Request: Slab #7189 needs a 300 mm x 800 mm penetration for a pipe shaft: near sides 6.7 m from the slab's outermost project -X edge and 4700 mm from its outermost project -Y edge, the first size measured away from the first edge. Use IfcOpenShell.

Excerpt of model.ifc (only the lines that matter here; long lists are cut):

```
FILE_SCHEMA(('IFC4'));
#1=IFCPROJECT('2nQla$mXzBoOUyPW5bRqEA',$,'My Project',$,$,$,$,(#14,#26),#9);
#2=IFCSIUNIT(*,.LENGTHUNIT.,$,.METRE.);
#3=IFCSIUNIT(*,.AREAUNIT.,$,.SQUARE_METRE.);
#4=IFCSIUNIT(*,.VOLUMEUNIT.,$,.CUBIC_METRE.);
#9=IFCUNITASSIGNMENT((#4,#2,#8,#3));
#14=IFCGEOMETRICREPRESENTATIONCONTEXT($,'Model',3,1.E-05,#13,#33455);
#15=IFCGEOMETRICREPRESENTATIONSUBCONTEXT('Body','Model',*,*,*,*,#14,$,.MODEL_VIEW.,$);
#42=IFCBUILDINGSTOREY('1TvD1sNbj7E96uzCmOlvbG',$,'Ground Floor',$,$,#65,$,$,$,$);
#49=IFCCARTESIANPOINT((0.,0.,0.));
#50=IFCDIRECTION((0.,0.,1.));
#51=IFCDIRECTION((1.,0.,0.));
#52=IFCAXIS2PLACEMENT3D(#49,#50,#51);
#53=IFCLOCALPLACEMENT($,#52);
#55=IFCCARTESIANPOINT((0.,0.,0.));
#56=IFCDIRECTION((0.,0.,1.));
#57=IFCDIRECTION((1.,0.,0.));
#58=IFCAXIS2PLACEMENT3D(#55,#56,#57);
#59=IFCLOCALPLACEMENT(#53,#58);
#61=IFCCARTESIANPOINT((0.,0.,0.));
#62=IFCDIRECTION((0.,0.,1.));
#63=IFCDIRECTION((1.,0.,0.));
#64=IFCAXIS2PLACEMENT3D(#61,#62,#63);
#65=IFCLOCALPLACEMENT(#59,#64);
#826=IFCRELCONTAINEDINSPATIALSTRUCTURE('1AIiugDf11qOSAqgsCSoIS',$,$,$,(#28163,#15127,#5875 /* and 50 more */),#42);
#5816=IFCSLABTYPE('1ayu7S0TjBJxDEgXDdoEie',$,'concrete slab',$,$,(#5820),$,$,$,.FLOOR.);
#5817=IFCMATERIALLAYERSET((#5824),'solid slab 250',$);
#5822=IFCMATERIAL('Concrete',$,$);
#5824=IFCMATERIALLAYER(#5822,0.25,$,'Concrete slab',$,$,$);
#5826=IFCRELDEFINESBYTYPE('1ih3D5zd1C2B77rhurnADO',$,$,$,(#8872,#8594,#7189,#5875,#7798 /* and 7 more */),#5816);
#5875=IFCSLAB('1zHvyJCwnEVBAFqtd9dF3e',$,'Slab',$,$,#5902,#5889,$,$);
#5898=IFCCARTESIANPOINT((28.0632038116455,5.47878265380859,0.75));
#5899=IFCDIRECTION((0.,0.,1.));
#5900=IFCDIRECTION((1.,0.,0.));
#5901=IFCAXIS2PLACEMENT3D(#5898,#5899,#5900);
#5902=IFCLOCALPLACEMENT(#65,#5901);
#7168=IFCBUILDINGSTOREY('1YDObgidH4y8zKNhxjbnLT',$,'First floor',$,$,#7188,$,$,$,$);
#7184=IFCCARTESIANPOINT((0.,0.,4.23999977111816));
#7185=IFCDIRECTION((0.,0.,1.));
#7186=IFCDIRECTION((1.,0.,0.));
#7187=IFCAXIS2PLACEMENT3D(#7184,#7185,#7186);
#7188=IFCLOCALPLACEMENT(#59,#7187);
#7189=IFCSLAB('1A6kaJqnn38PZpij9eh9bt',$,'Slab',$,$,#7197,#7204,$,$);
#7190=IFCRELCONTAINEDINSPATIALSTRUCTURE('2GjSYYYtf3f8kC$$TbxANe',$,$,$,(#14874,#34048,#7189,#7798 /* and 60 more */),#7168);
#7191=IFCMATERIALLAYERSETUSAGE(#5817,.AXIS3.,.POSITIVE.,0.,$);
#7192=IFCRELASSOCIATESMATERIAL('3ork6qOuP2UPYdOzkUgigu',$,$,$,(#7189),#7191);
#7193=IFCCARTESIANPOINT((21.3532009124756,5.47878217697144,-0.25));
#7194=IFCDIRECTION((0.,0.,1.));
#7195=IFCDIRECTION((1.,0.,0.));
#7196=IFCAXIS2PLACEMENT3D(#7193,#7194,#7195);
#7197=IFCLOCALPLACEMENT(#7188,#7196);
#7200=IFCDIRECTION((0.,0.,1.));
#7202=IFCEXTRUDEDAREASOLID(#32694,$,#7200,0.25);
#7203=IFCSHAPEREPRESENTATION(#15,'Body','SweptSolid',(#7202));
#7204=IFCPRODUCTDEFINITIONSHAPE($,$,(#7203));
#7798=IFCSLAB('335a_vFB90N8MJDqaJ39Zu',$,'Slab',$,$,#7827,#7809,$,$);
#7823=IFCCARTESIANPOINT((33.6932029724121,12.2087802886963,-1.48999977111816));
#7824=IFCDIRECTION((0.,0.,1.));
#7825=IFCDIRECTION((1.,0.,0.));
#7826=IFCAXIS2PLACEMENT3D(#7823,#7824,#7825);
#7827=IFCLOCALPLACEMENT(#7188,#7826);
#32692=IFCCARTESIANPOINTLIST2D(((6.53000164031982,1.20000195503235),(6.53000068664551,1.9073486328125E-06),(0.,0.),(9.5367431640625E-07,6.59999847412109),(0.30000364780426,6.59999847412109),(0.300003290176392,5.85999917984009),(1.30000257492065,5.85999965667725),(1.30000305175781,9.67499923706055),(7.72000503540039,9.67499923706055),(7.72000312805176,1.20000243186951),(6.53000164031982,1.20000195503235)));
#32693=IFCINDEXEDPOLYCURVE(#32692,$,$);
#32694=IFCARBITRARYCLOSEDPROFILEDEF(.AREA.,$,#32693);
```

```python
import numpy as np
import ifcopenshell
import ifcopenshell.api.feature
import ifcopenshell.api.geometry
import ifcopenshell.api.root
import ifcopenshell.geom
import ifcopenshell.util.placement
import ifcopenshell.util.representation
import ifcopenshell.util.shape
import ifcopenshell.util.unit

model = ifcopenshell.open("model.ifc")
unit_scale = ifcopenshell.util.unit.calculate_unit_scale(model)
settings = ifcopenshell.geom.settings()


def volume(element):
    """Net volume in cubic metres, openings subtracted."""
    shape = ifcopenshell.geom.create_shape(settings, element)
    return ifcopenshell.util.shape.get_volume(shape.geometry)


slab = model.by_id(7189)
before = volume(slab)

# Extent in the slab's own axes, in metres. The edges named are its -X and -Y sides.
slab_shape = ifcopenshell.geom.create_shape(settings, slab)
vertices = ifcopenshell.util.shape.get_vertices(slab_shape.geometry)
x_min, y_min, bottom = vertices.min(axis=0)
top = vertices[:, 2].max()

opening = ifcopenshell.api.root.create_entity(model, ifc_class="IfcOpeningElement", name="Pipe shaft opening", predefined_type="OPENING")
context = ifcopenshell.util.representation.get_context(model, "Model", "Body", "MODEL_VIEW")
width, depth = 0.3, 0.8
outline = [(0.0, 0.0), (width, 0.0), (width, depth), (0.0, depth), (0.0, 0.0)]
# Overshoot both faces by 50 mm so the cut is clean.
shape = ifcopenshell.api.geometry.add_slab_representation(
    model, context=context, depth=top - bottom + 0.1, polyline=outline
)
ifcopenshell.api.geometry.assign_representation(model, product=opening, representation=shape)

matrix = ifcopenshell.util.placement.get_local_placement(slab.ObjectPlacement)
matrix[:, 3] = matrix @ np.append(np.array([x_min + 6.7, y_min + 4.7, bottom - 0.05]) / unit_scale, 1.0)
ifcopenshell.api.geometry.edit_object_placement(model, product=opening, matrix=matrix, is_si=False)
ifcopenshell.api.feature.add_feature(model, feature=opening, element=slab)

after = volume(slab)

print(f"slab volume {before:.3f} -> {after:.3f} m3")

model.write("model_v2.ifc")
```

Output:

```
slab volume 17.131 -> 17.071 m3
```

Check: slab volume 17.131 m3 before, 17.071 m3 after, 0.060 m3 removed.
